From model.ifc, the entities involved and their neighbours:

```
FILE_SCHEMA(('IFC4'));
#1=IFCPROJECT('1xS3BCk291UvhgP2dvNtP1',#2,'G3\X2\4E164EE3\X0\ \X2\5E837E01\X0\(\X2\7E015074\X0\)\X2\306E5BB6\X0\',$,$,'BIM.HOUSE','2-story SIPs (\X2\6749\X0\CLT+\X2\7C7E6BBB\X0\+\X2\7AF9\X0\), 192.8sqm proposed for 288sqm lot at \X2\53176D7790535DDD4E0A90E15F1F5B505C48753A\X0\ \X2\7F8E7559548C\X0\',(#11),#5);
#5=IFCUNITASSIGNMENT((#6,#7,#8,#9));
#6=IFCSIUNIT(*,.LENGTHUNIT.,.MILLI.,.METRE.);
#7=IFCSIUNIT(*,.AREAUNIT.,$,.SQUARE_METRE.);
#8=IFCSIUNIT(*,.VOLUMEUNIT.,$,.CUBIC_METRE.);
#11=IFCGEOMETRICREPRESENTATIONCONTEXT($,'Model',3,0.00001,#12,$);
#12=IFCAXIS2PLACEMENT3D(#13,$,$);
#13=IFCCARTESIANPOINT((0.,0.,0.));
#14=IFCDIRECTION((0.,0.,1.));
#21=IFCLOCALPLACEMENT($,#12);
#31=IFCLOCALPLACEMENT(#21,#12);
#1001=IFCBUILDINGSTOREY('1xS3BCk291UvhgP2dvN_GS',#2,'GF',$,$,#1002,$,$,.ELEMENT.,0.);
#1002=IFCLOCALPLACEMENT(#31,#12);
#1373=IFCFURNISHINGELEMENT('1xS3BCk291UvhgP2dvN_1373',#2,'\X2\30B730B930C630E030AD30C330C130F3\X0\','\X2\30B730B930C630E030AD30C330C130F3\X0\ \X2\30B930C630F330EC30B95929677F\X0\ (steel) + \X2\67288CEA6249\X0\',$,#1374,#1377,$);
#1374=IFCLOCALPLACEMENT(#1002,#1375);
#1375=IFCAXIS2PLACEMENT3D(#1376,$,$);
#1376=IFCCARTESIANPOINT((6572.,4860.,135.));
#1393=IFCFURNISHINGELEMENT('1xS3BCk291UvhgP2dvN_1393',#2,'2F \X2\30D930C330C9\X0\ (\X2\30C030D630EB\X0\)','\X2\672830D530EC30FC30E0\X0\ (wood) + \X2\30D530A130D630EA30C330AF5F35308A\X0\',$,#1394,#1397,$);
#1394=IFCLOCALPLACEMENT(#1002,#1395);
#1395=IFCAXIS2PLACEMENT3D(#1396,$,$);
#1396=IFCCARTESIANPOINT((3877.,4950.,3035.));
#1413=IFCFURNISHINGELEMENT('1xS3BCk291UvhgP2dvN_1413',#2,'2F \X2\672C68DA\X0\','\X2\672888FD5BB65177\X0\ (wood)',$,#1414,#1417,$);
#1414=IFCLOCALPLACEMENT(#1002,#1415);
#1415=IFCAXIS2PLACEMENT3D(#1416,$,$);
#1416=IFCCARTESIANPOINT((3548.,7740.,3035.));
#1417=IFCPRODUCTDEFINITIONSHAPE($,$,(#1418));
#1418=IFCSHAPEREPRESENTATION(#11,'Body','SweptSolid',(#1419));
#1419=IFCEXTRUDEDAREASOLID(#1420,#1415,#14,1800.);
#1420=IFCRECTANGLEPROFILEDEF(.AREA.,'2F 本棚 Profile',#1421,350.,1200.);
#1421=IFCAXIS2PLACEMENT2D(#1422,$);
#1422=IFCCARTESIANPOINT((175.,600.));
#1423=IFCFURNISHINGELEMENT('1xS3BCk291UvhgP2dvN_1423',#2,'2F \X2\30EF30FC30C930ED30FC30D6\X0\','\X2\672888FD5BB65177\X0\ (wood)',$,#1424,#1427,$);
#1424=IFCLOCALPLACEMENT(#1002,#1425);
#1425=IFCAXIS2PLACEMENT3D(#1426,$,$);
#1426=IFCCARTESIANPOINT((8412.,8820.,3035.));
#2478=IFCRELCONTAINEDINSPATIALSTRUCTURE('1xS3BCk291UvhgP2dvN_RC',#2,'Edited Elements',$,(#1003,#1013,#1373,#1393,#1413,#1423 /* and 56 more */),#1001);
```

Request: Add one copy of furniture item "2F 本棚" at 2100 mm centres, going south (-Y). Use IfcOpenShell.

```python
import numpy as np
import ifcopenshell
import ifcopenshell.api.geometry
import ifcopenshell.api.root
import ifcopenshell.util.element
import ifcopenshell.util.placement
import ifcopenshell.util.unit

model = ifcopenshell.open("model.ifc")
unit_scale = ifcopenshell.util.unit.calculate_unit_scale(model)


def reuse_history(source, copy):
    """copy_class also copies each property set's owner history, people and application; keep the originals."""
    for rel in copy.IsDefinedBy:
        if rel.is_a("IfcRelDefinesByProperties") and (history := rel.RelatingPropertyDefinition.OwnerHistory):
            rel.RelatingPropertyDefinition.OwnerHistory = source.OwnerHistory
            ifcopenshell.util.element.remove_deep2(model, history)


source = model.by_id(1413)
base = ifcopenshell.util.placement.get_local_placement(source.ObjectPlacement)
step = np.array([0.0, -1.0, 0.0]) * 2.1 / unit_scale

for i in range(1, 2):
    copy = ifcopenshell.api.root.copy_class(model, product=source)
    copy.Representation = ifcopenshell.util.element.copy_deep(
        model, source.Representation, exclude=["IfcGeometricRepresentationContext", "IfcRepresentationMap"]
    )
    reuse_history(source, copy)
    matrix = base.copy()
    matrix[:3, 3] += i * step
    print("added at", matrix[:3, 3].round(3) + 0.0)
    ifcopenshell.api.geometry.edit_object_placement(model, product=copy, matrix=matrix, is_si=False)

model.write("model_rev.ifc")
```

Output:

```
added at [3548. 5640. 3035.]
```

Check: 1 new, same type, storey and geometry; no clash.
